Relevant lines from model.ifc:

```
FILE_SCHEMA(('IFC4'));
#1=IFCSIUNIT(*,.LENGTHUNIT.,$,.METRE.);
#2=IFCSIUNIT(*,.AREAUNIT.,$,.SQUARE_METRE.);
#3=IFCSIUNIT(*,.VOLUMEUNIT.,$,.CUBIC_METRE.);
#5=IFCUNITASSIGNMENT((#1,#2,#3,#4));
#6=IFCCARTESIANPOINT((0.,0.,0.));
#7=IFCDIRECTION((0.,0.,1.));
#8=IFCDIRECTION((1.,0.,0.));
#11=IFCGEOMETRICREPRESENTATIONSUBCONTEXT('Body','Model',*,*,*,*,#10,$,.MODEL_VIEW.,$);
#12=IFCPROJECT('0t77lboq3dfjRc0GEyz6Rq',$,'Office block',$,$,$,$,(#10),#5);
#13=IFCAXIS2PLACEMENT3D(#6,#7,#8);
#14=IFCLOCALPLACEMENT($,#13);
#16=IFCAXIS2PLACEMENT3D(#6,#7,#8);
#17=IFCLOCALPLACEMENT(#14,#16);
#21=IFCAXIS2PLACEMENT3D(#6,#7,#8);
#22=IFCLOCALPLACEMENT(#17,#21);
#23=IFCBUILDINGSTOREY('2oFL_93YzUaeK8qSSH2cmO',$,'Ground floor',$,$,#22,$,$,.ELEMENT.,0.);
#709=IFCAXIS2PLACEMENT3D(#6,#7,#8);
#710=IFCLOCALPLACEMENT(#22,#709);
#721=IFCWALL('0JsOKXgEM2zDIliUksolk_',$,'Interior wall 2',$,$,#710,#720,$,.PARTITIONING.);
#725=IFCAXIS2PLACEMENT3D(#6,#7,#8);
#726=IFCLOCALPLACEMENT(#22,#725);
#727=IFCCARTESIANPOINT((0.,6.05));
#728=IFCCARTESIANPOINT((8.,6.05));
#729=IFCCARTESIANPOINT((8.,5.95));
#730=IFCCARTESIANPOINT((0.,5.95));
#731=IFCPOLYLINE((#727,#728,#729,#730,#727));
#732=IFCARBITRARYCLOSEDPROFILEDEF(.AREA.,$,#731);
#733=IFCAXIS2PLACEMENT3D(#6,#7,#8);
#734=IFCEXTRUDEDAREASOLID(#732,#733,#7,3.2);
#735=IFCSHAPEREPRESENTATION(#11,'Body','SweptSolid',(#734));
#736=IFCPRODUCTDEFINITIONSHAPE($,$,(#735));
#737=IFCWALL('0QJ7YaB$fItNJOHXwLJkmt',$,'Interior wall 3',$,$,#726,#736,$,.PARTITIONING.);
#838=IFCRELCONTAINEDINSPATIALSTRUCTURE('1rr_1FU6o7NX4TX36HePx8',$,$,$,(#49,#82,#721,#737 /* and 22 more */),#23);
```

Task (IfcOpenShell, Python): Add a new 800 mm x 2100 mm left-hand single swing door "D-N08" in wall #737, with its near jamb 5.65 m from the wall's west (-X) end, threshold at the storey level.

```python
import numpy as np
import ifcopenshell
import ifcopenshell.api.feature
import ifcopenshell.api.geometry
import ifcopenshell.api.root
import ifcopenshell.api.spatial
import ifcopenshell.geom
import ifcopenshell.util.element
import ifcopenshell.util.placement
import ifcopenshell.util.representation
import ifcopenshell.util.shape
import ifcopenshell.util.unit

model = ifcopenshell.open("model.ifc")
unit_scale = ifcopenshell.util.unit.calculate_unit_scale(model)
settings = ifcopenshell.geom.settings()


def volume(element):
    """Net volume in cubic metres, openings subtracted."""
    shape = ifcopenshell.geom.create_shape(settings, element)
    return ifcopenshell.util.shape.get_volume(shape.geometry)


wall = model.by_guid("0QJ7YaB$fItNJOHXwLJkmt")
storey = ifcopenshell.util.element.get_container(wall, ifc_class="IfcBuildingStorey")
context = ifcopenshell.util.representation.get_context(model, "Model", "Body", "MODEL_VIEW")
before = volume(wall)

width, height, from_end, sill = 0.8, 2.1, 5.65, 0.0  # metres

# The wall runs along its own X axis, and the end named is its -X end.
wall_shape = ifcopenshell.geom.create_shape(settings, wall)
x, y, z = ifcopenshell.util.shape.get_vertices(wall_shape.geometry).T
start = x.min() + from_end
face, thickness = float(y.min()), float(y.max() - y.min())
wall_matrix = ifcopenshell.util.placement.get_local_placement(wall.ObjectPlacement)
level = ifcopenshell.util.placement.get_local_placement(storey.ObjectPlacement)[2, 3]


def in_wall(x, y):
    """Placement at x, y metres in the wall's axes, at sill height."""
    matrix = wall_matrix.copy()
    matrix[:, 3] = wall_matrix @ np.array([x / unit_scale, y / unit_scale, 0.0, 1.0])
    matrix[2, 3] = level + sill / unit_scale
    return matrix


# Opening: a box that overshoots both wall faces by 50 mm.
opening = ifcopenshell.api.root.create_entity(model, ifc_class="IfcOpeningElement", predefined_type="OPENING")
box = ifcopenshell.api.geometry.add_wall_representation(
    model, context=context, length=width, height=height, thickness=thickness + 0.1
)
ifcopenshell.api.geometry.assign_representation(model, product=opening, representation=box)
ifcopenshell.api.geometry.edit_object_placement(model, product=opening, matrix=in_wall(start, face - 0.05), is_si=False)
ifcopenshell.api.feature.add_feature(model, feature=opening, element=wall)

door = ifcopenshell.api.root.create_entity(model, ifc_class="IfcDoor", name="D-N08", predefined_type="DOOR")
door.OverallWidth, door.OverallHeight = width / unit_scale, height / unit_scale
door.OperationType = "SINGLE_SWING_LEFT"
body = ifcopenshell.api.geometry.add_door_representation(
    model,
    context=context,
    overall_width=door.OverallWidth,
    overall_height=door.OverallHeight,
    operation_type="SINGLE_SWING_LEFT",
    lining_properties={"LiningDepth": thickness / unit_scale, "ThresholdDepth": thickness / unit_scale},
)
ifcopenshell.api.geometry.assign_representation(model, product=door, representation=body)
ifcopenshell.api.spatial.assign_container(model, products=[door], relating_structure=storey)
ifcopenshell.api.feature.add_filling(model, opening=opening, element=door)

# The lining spans the wall, so the door starts at the wall face.
ifcopenshell.api.geometry.edit_object_placement(model, product=door, matrix=in_wall(start, face), is_si=False)

after = volume(wall)

print(f"wall volume {before:.3f} -> {after:.3f} m3")

model.write("model_edited.ifc")
```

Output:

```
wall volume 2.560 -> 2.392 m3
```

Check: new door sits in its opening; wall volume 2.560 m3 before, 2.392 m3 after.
